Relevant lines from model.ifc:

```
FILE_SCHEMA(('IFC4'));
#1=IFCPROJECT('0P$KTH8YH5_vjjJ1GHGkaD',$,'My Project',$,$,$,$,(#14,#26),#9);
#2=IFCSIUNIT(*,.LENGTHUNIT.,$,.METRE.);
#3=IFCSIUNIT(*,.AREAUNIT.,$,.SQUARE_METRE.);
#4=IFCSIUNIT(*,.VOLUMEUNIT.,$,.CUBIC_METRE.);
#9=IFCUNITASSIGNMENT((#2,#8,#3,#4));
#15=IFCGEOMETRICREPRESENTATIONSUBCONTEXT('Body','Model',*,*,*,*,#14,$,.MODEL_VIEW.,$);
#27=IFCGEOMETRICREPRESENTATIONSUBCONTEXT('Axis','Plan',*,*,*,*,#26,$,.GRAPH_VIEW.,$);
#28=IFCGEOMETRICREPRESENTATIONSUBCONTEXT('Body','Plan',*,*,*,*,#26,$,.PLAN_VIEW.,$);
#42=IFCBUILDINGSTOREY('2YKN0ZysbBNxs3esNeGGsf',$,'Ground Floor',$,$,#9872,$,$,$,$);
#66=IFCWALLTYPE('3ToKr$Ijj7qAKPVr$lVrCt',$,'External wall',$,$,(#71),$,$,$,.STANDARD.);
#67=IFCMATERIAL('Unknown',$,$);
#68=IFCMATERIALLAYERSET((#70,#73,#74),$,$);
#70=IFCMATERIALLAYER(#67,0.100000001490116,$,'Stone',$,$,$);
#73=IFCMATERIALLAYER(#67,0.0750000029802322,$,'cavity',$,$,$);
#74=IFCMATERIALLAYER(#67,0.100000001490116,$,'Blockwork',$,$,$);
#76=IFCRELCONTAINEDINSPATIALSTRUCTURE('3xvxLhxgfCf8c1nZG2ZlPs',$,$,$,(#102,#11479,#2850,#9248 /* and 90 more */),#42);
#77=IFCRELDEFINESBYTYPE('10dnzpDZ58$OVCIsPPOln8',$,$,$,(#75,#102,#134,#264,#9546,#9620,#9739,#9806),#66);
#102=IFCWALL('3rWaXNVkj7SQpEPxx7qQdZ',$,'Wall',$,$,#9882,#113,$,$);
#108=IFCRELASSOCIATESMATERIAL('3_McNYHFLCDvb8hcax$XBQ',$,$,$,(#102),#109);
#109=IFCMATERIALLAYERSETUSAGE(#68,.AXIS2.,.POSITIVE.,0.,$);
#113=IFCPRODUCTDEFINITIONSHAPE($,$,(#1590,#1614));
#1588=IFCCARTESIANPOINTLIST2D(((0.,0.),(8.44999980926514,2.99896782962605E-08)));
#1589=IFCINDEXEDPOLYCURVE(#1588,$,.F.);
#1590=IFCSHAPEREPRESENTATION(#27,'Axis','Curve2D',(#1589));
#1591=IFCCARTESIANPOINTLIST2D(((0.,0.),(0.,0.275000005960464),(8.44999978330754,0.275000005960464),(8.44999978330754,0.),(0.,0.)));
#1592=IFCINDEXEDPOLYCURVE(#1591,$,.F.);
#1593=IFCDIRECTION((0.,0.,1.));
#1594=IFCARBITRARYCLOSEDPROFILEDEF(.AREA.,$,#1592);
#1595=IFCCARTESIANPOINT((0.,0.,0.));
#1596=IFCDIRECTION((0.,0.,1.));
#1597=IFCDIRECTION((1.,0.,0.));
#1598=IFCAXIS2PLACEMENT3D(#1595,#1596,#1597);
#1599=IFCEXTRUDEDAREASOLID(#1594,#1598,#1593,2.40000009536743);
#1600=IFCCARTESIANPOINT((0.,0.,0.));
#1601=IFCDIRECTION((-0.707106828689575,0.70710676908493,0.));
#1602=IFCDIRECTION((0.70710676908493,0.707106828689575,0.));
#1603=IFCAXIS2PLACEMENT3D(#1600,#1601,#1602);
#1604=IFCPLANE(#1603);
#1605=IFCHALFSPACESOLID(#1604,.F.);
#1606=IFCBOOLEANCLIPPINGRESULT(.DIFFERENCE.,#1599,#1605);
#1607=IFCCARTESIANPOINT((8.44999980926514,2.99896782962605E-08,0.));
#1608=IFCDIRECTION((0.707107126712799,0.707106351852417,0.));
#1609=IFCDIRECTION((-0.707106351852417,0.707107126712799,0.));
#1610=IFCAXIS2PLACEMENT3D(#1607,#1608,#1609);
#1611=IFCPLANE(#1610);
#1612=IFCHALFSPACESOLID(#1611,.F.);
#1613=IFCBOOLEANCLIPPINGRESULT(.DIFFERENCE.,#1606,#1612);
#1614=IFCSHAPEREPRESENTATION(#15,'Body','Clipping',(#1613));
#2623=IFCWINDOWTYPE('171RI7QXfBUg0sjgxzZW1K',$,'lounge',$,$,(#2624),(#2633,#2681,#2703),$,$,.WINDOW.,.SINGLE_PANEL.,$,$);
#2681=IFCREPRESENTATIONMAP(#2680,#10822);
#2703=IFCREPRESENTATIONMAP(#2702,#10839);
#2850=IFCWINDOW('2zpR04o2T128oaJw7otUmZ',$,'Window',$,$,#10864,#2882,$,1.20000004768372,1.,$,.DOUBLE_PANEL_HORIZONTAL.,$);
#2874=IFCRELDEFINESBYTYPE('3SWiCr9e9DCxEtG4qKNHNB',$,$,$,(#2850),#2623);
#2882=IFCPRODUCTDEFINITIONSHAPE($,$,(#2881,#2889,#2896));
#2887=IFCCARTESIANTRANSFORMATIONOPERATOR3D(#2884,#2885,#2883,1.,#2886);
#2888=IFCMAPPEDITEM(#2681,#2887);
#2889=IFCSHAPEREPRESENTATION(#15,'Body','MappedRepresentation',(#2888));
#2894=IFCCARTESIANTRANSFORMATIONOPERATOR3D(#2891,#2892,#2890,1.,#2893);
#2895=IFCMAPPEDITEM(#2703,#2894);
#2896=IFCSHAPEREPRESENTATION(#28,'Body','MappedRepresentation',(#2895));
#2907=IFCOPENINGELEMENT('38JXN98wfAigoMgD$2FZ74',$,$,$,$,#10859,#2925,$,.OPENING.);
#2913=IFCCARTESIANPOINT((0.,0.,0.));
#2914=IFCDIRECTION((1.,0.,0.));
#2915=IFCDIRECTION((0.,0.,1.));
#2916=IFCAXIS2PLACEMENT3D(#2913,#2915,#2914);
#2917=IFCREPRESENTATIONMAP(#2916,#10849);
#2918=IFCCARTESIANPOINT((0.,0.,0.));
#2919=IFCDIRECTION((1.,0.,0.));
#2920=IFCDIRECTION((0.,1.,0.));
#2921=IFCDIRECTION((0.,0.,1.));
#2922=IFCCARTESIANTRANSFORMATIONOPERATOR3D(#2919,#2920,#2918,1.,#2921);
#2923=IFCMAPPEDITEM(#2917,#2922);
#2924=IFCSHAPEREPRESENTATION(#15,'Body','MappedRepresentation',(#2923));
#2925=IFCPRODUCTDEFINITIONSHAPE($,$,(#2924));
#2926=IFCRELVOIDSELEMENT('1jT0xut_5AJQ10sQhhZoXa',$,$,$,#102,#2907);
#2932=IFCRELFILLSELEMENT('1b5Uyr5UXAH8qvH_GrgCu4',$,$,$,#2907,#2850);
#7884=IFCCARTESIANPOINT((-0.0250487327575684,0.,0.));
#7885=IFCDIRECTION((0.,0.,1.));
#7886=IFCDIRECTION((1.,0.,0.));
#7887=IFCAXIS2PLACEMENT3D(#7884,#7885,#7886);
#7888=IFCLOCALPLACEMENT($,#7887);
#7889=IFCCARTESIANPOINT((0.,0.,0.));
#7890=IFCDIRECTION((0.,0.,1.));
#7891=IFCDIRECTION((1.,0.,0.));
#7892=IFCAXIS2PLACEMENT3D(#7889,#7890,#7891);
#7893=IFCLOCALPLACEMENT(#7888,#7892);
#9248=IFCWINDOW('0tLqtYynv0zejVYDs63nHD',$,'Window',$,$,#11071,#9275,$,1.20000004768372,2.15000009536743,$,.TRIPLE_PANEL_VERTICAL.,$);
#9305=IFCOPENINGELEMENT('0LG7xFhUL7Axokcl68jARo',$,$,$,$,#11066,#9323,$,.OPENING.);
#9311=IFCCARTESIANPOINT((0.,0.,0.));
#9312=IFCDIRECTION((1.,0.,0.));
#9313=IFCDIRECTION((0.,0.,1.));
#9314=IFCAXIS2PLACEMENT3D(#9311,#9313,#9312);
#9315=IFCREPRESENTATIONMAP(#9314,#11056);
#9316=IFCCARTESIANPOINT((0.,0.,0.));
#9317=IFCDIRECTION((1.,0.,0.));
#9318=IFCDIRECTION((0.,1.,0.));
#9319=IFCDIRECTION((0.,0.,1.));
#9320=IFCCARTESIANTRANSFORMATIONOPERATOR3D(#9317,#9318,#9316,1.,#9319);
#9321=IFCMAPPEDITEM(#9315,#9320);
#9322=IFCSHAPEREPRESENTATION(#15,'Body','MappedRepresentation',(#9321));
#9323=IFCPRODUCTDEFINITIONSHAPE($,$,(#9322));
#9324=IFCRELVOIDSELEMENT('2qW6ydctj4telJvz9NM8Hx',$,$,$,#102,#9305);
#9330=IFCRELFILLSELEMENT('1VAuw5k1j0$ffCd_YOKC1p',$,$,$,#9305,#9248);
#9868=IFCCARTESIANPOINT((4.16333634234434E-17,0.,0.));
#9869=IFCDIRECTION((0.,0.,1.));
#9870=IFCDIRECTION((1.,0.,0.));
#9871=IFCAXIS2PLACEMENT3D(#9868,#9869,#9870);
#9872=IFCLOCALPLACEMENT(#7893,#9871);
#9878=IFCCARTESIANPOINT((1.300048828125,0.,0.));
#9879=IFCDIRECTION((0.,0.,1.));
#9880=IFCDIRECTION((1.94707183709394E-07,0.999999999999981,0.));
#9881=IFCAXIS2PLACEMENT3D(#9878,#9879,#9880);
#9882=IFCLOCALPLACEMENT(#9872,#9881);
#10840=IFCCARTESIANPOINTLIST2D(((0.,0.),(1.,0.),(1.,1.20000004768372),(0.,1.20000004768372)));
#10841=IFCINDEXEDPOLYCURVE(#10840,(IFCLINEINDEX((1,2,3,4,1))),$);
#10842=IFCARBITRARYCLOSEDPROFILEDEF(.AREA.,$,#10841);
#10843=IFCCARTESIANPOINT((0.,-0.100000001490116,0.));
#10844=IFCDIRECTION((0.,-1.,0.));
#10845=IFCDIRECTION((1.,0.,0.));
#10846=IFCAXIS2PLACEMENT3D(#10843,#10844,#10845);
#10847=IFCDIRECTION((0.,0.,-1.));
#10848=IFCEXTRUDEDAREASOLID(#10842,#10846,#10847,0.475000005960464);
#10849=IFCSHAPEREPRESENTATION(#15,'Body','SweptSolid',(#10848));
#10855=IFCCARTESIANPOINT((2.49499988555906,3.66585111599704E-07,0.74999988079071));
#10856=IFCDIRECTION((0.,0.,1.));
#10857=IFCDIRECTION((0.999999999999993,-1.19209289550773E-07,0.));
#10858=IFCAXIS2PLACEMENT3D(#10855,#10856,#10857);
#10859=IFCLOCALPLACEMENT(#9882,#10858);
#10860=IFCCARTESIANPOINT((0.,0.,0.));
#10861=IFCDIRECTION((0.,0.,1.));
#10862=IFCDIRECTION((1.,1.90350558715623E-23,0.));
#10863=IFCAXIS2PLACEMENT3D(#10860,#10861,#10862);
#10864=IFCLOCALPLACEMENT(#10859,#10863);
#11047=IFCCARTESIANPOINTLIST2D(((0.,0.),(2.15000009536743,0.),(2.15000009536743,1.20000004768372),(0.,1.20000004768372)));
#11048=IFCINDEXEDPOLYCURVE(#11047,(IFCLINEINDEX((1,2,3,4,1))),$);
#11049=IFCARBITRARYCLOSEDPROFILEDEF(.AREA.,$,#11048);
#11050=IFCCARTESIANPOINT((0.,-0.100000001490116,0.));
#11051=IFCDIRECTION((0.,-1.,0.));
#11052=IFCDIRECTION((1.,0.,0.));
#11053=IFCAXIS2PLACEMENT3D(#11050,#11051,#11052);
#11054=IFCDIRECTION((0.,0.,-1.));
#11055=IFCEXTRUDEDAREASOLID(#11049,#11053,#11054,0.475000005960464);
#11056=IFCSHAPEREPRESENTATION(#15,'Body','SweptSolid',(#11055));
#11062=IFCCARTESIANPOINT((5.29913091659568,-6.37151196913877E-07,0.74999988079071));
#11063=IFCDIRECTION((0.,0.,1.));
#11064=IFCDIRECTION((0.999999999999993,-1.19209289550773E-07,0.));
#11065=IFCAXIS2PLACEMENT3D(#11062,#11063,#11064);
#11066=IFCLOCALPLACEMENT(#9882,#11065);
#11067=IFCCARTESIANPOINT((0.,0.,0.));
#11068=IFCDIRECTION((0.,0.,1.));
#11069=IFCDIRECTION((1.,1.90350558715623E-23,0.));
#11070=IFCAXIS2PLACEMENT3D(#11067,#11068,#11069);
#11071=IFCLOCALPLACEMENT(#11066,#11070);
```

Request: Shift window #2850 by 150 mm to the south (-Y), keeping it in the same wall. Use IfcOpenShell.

```python
import ifcopenshell
import ifcopenshell.api.geometry
import ifcopenshell.util.placement

model = ifcopenshell.open("model.ifc")

window = model.by_guid("2zpR04o2T128oaJw7otUmZ")
opening = window.FillsVoids[0].RelatingOpeningElement
wall = opening.VoidsElements[0].RelatingBuildingElement

wall_matrix = ifcopenshell.util.placement.get_local_placement(wall.ObjectPlacement)
shift = wall_matrix[:3, 0] * -0.15
before = ifcopenshell.util.placement.get_local_placement(window.ObjectPlacement)[:3, 3].copy()

# The window is placed relative to its opening, so it follows when the opening moves.
matrix = ifcopenshell.util.placement.get_local_placement(opening.ObjectPlacement)
matrix[:3, 3] += shift
ifcopenshell.api.geometry.edit_object_placement(
    model, product=opening, matrix=matrix, is_si=False, should_transform_children=True
)

after = ifcopenshell.util.placement.get_local_placement(window.ObjectPlacement)[:3, 3]
print("window moved by", (after - before).round(3) + 0.0)

model.write("model-out.ifc")
```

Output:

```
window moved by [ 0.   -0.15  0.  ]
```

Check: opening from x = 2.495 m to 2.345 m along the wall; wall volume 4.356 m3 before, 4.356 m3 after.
